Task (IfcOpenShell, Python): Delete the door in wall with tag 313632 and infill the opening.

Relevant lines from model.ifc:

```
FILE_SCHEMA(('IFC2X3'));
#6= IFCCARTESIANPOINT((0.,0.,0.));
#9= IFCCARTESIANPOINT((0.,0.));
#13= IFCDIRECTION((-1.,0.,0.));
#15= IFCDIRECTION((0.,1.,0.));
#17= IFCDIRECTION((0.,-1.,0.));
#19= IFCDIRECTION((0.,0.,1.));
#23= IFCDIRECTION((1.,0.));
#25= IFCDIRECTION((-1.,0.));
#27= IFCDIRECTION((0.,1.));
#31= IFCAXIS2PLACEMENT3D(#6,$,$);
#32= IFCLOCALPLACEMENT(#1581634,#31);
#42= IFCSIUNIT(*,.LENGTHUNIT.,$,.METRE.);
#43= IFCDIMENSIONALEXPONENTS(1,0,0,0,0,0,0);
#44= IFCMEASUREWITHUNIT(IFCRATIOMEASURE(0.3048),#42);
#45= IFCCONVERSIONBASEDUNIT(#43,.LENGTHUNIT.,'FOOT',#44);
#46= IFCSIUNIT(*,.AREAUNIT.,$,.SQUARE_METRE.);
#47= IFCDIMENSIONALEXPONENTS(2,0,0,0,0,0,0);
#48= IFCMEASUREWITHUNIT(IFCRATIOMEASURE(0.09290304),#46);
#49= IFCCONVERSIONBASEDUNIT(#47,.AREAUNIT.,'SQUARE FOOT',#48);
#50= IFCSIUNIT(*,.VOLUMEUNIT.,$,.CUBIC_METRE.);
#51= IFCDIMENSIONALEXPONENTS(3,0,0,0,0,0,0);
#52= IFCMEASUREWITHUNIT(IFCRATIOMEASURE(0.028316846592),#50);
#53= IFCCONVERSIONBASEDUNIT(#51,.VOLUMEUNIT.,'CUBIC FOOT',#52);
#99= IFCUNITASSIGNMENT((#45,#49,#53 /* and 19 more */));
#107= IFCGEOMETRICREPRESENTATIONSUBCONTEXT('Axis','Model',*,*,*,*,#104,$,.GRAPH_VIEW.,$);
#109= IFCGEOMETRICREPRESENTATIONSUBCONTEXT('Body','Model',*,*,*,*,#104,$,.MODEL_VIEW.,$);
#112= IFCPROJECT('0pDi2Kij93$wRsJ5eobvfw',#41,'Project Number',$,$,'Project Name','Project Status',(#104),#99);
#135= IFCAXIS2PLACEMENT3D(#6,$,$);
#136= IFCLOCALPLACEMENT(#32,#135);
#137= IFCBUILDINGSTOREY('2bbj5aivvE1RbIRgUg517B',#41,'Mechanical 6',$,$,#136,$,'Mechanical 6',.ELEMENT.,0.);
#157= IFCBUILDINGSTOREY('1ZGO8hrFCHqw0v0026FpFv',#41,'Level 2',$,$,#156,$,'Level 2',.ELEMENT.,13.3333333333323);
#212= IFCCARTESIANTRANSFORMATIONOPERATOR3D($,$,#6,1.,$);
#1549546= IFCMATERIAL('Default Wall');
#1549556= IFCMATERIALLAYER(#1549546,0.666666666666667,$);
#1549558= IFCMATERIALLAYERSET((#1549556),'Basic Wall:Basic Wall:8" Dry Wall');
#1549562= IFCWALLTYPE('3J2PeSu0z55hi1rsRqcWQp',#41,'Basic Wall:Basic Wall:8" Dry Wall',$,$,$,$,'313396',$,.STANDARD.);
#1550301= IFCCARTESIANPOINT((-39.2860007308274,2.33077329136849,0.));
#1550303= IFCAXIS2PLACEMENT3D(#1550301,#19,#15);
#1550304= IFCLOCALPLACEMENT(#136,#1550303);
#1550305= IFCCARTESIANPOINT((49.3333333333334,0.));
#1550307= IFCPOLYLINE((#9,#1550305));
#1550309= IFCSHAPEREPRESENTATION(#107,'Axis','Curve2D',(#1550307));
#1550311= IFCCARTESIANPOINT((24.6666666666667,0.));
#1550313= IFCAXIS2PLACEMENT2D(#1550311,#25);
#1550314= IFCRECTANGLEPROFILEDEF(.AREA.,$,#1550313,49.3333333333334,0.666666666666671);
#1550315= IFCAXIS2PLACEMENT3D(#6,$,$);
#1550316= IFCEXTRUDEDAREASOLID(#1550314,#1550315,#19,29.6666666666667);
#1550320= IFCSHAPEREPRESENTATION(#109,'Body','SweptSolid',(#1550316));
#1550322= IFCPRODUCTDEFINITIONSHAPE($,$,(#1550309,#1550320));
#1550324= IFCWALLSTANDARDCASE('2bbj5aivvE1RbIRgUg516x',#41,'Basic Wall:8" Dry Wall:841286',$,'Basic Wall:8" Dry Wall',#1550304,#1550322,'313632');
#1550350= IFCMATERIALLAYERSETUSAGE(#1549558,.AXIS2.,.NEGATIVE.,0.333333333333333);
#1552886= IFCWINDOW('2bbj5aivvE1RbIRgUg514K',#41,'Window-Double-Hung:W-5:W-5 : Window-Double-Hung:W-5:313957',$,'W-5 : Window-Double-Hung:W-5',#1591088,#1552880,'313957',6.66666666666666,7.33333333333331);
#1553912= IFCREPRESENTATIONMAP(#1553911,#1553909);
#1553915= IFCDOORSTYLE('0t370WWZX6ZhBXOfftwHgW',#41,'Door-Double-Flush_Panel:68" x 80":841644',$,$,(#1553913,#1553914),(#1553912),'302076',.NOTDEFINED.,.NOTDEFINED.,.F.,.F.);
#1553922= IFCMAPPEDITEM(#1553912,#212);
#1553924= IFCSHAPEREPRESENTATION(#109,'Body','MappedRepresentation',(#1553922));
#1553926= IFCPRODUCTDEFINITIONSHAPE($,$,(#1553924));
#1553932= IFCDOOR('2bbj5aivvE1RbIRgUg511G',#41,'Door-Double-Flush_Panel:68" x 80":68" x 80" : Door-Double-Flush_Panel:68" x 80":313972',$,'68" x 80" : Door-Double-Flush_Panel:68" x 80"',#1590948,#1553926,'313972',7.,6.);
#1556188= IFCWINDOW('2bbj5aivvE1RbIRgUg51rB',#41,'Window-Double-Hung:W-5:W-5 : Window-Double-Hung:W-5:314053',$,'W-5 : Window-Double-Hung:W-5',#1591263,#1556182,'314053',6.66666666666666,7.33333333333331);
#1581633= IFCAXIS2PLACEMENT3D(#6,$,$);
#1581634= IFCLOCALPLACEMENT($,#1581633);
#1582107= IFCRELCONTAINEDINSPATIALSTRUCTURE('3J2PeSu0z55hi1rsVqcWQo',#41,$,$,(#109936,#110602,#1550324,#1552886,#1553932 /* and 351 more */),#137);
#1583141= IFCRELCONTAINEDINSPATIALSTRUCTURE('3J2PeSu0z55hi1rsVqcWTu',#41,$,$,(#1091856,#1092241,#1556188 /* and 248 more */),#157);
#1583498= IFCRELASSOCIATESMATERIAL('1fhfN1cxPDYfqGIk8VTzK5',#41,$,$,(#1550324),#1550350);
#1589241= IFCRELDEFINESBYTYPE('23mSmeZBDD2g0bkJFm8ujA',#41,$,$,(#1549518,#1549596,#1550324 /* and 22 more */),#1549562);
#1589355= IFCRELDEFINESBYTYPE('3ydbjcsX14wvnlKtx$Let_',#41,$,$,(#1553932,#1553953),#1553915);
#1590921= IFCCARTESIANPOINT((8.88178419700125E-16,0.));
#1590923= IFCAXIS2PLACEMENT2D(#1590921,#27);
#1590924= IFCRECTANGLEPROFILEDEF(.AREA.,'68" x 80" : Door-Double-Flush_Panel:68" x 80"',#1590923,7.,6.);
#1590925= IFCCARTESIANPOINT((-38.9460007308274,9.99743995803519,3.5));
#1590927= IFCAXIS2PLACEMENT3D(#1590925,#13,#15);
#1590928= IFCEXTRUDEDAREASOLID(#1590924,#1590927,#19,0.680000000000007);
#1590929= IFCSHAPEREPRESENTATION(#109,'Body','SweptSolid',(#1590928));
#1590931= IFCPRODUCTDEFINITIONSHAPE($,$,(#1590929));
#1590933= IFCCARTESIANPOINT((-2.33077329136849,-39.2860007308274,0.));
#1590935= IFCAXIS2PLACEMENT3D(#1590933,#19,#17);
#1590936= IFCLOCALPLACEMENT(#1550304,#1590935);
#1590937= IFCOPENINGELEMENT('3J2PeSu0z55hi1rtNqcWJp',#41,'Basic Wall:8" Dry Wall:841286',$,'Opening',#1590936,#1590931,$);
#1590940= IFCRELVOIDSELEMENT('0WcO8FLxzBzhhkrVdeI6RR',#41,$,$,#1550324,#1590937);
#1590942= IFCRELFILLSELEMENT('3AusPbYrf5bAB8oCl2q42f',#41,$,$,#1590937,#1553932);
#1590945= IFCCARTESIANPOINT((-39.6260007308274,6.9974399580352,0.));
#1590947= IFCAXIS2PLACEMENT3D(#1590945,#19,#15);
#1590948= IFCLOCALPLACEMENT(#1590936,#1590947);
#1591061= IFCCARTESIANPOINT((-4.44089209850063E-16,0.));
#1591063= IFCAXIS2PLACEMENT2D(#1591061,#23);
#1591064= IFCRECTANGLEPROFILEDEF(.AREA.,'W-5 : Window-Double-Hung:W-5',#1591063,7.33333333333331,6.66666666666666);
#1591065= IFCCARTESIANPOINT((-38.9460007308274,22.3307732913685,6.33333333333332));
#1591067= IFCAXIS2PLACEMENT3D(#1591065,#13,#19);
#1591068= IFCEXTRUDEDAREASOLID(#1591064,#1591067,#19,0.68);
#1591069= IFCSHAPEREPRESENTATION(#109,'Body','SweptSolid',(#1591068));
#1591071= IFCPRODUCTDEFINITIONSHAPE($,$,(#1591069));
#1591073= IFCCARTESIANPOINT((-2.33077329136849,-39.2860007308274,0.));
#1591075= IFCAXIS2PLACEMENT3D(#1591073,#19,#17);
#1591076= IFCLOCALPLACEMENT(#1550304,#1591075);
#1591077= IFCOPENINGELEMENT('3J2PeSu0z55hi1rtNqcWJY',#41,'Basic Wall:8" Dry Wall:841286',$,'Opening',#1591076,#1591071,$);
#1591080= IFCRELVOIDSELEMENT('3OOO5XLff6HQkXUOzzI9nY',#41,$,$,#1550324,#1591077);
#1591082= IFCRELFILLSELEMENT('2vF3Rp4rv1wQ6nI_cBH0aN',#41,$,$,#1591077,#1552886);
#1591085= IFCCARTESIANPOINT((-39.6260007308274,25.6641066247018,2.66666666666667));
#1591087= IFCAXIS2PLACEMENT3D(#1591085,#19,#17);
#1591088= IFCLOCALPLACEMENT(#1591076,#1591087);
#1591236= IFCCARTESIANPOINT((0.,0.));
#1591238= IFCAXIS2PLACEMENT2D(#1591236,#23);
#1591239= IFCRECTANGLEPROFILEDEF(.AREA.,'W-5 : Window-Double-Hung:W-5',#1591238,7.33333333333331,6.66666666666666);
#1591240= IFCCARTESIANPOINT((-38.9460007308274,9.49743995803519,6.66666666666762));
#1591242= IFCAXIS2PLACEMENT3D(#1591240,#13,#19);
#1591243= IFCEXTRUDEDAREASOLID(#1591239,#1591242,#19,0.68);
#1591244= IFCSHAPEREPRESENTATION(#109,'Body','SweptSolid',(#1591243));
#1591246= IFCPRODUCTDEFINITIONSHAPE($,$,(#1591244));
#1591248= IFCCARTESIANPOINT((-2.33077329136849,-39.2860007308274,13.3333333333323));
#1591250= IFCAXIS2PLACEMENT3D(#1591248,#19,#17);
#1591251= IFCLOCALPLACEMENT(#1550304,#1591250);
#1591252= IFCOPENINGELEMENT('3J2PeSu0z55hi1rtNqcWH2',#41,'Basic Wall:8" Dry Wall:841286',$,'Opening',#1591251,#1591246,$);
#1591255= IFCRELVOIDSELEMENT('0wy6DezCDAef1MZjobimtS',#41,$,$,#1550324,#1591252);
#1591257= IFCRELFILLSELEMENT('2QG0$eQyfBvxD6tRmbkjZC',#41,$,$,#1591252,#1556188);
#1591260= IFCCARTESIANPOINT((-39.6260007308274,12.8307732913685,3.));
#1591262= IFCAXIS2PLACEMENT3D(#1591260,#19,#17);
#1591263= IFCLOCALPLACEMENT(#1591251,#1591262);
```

```python
import ifcopenshell
import ifcopenshell.api.feature
import ifcopenshell.api.root
import ifcopenshell.geom
import ifcopenshell.util.shape

model = ifcopenshell.open("model.ifc")
settings = ifcopenshell.geom.settings()


def volume(element):
    """Net volume in cubic metres, openings subtracted."""
    shape = ifcopenshell.geom.create_shape(settings, element)
    return ifcopenshell.util.shape.get_volume(shape.geometry)


door = model.by_id(1553932)
opening = door.FillsVoids[0].RelatingOpeningElement
wall = opening.VoidsElements[0].RelatingBuildingElement
before = volume(wall)

ifcopenshell.api.root.remove_product(model, product=door)
ifcopenshell.api.feature.remove_feature(model, feature=opening)

after = volume(wall)

print(f"wall volume {before:.3f} -> {after:.3f} m3")

model.write("model_updated.ifc")
```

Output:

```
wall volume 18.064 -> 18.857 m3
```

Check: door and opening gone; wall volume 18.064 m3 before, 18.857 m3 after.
